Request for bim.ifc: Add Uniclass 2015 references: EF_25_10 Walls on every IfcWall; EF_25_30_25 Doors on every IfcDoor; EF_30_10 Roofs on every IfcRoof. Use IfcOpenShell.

First a look at what the model holds.

```python
import ifcopenshell

model = ifcopenshell.open("bim.ifc")
print(model.schema)
print("classifications:", [c.Name for c in model.by_type("IfcClassification")])
for ifc_class in ("IfcDoor", "IfcRoof", "IfcStair", "IfcWall", "IfcWindow"):
    print(ifc_class, len(model.by_type(ifc_class)))
```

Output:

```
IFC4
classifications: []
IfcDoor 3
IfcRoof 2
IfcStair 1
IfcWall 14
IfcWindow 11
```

```python
import ifcopenshell
import ifcopenshell.api.classification

model = ifcopenshell.open("bim.ifc")

system = ifcopenshell.api.classification.add_classification(model, classification="Uniclass 2015")

codes = {
    "IfcWall": ("EF_25_10", "Walls"),
    "IfcDoor": ("EF_25_30_25", "Doors"),
    "IfcRoof": ("EF_30_10", "Roofs"),
}
for ifc_class, (code, name) in codes.items():
    products = model.by_type(ifc_class)
    ifcopenshell.api.classification.add_reference(
        model, products=products, classification=system, identification=code, name=name
    )
    print(code, len(products))

model.write("bim_edited.ifc")
```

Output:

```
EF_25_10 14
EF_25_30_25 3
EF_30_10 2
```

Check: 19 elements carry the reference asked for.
